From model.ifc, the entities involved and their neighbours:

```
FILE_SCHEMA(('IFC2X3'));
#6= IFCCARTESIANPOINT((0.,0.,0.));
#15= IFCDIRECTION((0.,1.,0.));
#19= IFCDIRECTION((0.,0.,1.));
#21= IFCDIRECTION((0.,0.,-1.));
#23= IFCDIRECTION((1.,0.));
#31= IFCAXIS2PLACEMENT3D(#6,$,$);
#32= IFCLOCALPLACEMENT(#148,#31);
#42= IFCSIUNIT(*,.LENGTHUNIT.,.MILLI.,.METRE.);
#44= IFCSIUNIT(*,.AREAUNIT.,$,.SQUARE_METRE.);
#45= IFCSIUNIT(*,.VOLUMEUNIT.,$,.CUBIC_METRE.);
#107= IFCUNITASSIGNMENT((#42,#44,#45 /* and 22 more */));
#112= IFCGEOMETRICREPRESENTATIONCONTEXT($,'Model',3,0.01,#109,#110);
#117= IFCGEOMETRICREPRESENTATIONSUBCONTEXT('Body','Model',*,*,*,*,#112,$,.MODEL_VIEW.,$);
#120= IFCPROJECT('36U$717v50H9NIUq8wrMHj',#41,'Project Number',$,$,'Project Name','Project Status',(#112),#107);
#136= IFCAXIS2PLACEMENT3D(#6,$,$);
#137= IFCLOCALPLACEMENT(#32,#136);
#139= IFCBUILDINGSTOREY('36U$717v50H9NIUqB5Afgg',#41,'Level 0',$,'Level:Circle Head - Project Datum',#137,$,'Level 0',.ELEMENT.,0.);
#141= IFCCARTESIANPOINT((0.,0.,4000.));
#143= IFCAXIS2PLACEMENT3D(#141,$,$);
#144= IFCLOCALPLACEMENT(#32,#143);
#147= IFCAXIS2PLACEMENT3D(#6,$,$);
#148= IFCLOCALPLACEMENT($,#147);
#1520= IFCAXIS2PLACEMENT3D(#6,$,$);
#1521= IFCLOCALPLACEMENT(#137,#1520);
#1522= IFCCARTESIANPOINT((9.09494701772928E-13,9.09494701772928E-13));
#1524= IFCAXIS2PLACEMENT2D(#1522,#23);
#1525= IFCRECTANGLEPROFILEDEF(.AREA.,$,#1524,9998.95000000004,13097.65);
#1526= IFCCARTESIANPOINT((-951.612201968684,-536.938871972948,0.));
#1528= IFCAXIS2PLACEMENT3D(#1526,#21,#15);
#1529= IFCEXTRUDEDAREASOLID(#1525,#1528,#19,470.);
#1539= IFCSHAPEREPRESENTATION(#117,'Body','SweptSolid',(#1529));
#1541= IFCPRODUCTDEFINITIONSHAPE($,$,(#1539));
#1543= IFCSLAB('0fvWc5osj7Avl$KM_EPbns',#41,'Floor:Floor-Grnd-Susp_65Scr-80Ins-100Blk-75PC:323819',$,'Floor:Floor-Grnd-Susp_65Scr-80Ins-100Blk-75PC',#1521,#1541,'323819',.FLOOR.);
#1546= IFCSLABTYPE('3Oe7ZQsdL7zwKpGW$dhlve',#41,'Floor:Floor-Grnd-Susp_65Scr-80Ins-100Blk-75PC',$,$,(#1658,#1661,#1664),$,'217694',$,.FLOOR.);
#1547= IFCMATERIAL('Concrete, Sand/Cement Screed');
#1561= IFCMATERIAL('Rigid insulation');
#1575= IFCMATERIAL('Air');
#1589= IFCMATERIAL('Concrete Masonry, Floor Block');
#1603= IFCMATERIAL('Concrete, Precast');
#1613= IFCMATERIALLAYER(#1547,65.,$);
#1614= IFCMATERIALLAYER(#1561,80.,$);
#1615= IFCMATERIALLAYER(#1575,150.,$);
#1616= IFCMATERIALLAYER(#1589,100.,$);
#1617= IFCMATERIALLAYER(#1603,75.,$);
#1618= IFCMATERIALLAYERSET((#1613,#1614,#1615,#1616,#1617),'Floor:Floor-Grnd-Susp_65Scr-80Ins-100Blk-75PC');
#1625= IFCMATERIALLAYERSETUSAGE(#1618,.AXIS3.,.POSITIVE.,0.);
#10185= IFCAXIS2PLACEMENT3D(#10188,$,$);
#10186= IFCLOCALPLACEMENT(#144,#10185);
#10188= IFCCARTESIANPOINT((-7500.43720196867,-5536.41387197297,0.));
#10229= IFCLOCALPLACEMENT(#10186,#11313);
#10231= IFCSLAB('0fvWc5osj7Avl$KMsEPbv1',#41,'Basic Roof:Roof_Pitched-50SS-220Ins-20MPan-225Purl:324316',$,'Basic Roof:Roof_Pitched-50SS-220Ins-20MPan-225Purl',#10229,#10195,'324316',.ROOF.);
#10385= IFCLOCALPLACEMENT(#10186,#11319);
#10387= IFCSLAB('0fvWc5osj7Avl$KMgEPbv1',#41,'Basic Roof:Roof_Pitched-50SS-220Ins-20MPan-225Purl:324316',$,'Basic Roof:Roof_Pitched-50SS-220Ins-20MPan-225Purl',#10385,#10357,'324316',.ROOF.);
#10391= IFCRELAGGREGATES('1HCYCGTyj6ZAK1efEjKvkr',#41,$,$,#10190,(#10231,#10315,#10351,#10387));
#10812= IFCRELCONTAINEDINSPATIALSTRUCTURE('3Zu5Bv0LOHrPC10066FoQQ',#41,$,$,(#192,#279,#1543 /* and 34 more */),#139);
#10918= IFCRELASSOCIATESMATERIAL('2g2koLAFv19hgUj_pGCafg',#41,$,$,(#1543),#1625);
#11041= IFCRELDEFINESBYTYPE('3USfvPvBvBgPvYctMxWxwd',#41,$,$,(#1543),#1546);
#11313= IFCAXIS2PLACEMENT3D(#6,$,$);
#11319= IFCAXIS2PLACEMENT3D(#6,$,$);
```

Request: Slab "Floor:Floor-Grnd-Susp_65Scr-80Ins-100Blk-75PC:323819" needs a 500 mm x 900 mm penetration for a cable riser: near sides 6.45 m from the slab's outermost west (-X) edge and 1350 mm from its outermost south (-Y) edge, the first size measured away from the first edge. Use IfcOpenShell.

```python
import numpy as np
import ifcopenshell
import ifcopenshell.api.feature
import ifcopenshell.api.geometry
import ifcopenshell.api.root
import ifcopenshell.geom
import ifcopenshell.util.placement
import ifcopenshell.util.representation
import ifcopenshell.util.shape
import ifcopenshell.util.unit

model = ifcopenshell.open("model.ifc")
unit_scale = ifcopenshell.util.unit.calculate_unit_scale(model)
settings = ifcopenshell.geom.settings()


def volume(element):
    """Net volume in cubic metres, openings subtracted."""
    shape = ifcopenshell.geom.create_shape(settings, element)
    return ifcopenshell.util.shape.get_volume(shape.geometry)


slab = model.by_id(1543)
before = volume(slab)

# Extent in the slab's own axes, in metres. The edges named are its -X and -Y sides.
slab_shape = ifcopenshell.geom.create_shape(settings, slab)
vertices = ifcopenshell.util.shape.get_vertices(slab_shape.geometry)
x_min, y_min, bottom = vertices.min(axis=0)
top = vertices[:, 2].max()

opening = ifcopenshell.api.root.create_entity(model, ifc_class="IfcOpeningElement", name="Cable riser opening")
context = ifcopenshell.util.representation.get_context(model, "Model", "Body", "MODEL_VIEW")
width, depth = 0.5, 0.9
outline = [(0.0, 0.0), (width, 0.0), (width, depth), (0.0, depth), (0.0, 0.0)]
# Overshoot both faces by 50 mm so the cut is clean.
shape = ifcopenshell.api.geometry.add_slab_representation(
    model, context=context, depth=top - bottom + 0.1, polyline=outline
)
ifcopenshell.api.geometry.assign_representation(model, product=opening, representation=shape)

matrix = ifcopenshell.util.placement.get_local_placement(slab.ObjectPlacement)
matrix[:, 3] = matrix @ np.append(np.array([x_min + 6.45, y_min + 1.35, bottom - 0.05]) / unit_scale, 1.0)
ifcopenshell.api.geometry.edit_object_placement(model, product=opening, matrix=matrix, is_si=False)
ifcopenshell.api.feature.add_feature(model, feature=opening, element=slab)

after = volume(slab)

print(f"slab volume {before:.3f} -> {after:.3f} m3")

model.write("model_rev.ifc")
```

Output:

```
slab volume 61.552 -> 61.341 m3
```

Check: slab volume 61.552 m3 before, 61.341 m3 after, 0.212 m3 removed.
